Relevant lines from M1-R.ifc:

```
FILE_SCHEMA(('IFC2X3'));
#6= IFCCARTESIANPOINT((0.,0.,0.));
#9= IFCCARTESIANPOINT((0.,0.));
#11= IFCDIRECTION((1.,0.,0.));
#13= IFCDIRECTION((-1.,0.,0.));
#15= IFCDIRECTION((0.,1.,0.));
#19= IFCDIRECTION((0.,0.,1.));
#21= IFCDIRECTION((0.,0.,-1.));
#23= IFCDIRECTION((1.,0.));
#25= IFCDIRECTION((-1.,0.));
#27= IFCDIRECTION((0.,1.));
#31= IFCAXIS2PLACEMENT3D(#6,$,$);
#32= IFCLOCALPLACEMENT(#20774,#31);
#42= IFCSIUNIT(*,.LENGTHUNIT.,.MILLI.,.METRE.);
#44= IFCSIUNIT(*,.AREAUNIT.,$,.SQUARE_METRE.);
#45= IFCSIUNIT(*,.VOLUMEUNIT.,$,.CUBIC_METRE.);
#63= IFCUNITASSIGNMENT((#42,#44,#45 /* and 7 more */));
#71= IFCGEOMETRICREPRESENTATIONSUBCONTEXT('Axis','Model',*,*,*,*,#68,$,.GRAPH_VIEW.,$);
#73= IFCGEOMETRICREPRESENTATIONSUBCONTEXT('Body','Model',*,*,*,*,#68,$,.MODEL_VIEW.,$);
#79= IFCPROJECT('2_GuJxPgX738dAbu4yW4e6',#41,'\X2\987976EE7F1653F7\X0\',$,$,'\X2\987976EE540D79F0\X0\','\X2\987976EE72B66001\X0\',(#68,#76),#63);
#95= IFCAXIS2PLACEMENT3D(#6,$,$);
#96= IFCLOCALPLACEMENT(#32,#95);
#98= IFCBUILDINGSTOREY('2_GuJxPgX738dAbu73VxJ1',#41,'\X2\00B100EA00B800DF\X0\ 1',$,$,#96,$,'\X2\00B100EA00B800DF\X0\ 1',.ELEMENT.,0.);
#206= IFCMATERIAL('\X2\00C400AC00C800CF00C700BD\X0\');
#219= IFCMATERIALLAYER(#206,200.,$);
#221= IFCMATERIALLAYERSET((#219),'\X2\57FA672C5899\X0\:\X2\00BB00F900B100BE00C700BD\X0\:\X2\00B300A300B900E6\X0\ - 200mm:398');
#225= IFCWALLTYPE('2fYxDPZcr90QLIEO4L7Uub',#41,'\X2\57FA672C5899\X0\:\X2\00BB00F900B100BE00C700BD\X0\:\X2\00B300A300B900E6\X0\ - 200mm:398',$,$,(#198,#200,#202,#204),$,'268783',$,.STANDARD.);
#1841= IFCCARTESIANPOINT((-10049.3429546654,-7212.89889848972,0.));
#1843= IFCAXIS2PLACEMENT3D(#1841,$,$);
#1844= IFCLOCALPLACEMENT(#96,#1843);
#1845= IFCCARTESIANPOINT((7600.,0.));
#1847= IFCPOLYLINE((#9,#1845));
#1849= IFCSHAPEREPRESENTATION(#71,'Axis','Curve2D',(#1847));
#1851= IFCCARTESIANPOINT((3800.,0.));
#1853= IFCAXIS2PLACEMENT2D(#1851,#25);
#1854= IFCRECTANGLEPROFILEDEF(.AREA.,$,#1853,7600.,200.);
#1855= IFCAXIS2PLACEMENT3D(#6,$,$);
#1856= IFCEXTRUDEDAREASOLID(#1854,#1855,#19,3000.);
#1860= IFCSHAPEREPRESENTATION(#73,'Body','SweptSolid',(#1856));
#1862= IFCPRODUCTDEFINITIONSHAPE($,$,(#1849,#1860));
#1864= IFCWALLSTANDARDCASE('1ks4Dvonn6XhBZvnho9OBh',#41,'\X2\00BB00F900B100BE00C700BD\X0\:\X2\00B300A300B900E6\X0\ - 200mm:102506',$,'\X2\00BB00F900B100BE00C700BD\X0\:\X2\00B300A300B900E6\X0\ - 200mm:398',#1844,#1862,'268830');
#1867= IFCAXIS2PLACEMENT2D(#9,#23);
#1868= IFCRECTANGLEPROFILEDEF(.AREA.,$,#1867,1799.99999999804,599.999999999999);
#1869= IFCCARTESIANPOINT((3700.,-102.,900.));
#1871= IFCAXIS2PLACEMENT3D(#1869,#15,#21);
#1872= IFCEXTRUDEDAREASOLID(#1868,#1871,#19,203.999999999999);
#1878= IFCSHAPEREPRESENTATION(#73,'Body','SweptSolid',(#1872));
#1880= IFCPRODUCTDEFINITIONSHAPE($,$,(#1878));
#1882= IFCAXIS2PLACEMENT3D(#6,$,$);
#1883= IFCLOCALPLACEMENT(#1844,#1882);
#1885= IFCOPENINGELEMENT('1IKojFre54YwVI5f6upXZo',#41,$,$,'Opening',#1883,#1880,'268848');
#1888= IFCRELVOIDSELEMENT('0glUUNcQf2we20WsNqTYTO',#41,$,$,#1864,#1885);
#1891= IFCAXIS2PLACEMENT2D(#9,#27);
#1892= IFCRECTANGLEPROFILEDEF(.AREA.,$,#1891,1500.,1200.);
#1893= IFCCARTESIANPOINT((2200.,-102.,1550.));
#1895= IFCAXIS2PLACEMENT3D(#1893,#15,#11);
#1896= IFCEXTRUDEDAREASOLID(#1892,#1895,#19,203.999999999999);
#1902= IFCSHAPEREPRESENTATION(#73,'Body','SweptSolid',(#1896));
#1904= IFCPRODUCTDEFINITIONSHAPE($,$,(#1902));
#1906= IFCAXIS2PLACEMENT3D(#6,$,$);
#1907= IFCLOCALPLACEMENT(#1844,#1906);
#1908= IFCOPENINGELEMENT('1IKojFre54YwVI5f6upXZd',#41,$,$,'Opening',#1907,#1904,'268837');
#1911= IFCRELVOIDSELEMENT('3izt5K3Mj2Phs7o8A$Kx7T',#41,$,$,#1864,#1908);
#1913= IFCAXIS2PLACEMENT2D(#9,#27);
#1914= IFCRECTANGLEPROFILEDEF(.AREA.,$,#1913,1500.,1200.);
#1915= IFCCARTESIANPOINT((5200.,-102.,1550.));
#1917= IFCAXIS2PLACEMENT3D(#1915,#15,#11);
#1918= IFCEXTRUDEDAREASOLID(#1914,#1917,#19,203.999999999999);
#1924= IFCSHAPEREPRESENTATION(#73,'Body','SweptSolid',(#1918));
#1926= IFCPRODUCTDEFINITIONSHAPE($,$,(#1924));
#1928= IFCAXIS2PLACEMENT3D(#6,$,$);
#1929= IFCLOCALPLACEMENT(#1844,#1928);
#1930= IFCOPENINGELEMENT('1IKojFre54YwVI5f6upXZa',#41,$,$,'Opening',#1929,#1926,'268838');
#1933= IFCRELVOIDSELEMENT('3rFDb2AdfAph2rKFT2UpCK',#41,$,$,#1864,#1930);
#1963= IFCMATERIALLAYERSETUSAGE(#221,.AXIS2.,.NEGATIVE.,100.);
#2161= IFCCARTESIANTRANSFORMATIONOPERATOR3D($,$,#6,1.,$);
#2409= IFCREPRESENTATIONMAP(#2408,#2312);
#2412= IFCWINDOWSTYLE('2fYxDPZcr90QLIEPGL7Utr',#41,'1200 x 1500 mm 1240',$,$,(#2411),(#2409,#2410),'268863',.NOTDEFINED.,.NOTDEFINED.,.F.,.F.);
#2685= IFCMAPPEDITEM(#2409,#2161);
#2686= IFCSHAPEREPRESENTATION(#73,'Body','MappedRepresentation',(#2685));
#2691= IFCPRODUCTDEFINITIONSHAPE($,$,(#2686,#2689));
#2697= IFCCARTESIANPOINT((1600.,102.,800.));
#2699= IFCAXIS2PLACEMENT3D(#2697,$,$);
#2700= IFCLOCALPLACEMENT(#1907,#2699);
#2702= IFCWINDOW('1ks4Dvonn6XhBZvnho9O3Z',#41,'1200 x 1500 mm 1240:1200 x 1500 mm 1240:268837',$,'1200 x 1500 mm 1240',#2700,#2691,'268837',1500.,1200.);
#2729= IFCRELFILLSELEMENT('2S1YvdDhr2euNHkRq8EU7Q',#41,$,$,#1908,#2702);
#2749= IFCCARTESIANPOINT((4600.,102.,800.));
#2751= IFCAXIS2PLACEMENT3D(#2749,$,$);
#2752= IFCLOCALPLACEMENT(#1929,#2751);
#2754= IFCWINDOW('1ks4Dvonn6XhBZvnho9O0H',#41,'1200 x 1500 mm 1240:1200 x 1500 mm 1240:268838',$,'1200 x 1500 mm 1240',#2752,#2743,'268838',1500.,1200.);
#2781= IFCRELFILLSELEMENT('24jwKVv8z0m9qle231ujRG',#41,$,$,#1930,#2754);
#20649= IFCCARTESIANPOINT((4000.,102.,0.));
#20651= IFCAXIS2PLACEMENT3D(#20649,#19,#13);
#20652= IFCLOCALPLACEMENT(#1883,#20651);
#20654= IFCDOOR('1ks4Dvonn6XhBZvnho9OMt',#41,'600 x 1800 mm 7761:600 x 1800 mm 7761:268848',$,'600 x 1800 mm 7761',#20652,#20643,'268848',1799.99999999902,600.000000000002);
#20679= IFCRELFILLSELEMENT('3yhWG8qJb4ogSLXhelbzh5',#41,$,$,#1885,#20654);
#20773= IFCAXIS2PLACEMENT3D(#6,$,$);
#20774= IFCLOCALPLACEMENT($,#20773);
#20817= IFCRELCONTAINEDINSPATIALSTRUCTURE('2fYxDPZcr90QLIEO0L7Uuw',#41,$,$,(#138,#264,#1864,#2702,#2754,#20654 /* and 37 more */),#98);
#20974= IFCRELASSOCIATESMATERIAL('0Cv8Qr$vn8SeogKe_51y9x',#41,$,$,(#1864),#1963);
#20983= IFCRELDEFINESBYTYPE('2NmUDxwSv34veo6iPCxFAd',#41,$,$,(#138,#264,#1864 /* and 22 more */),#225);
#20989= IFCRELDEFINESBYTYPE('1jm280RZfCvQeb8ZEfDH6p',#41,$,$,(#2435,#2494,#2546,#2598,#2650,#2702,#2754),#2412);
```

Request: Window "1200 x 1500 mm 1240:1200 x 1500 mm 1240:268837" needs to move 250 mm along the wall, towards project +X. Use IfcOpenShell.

```python
import ifcopenshell
import ifcopenshell.api.geometry
import ifcopenshell.util.placement
import ifcopenshell.util.unit

model = ifcopenshell.open("M1-R.ifc")
unit_scale = ifcopenshell.util.unit.calculate_unit_scale(model)

window = model.by_id(2702)
opening = window.FillsVoids[0].RelatingOpeningElement
wall = opening.VoidsElements[0].RelatingBuildingElement

wall_matrix = ifcopenshell.util.placement.get_local_placement(wall.ObjectPlacement)
shift = wall_matrix[:3, 0] * 0.25 / unit_scale
before = ifcopenshell.util.placement.get_local_placement(window.ObjectPlacement)[:3, 3].copy()

# The window is placed relative to its opening, so it follows when the opening moves.
matrix = ifcopenshell.util.placement.get_local_placement(opening.ObjectPlacement)
matrix[:3, 3] += shift
ifcopenshell.api.geometry.edit_object_placement(
    model, product=opening, matrix=matrix, is_si=False, should_transform_children=True
)

after = ifcopenshell.util.placement.get_local_placement(window.ObjectPlacement)[:3, 3]
print("window moved by", (after - before).round(3) + 0.0)

model.write("M1-R_updated.ifc")
```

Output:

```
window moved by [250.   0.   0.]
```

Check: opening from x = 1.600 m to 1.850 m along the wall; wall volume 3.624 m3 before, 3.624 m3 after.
